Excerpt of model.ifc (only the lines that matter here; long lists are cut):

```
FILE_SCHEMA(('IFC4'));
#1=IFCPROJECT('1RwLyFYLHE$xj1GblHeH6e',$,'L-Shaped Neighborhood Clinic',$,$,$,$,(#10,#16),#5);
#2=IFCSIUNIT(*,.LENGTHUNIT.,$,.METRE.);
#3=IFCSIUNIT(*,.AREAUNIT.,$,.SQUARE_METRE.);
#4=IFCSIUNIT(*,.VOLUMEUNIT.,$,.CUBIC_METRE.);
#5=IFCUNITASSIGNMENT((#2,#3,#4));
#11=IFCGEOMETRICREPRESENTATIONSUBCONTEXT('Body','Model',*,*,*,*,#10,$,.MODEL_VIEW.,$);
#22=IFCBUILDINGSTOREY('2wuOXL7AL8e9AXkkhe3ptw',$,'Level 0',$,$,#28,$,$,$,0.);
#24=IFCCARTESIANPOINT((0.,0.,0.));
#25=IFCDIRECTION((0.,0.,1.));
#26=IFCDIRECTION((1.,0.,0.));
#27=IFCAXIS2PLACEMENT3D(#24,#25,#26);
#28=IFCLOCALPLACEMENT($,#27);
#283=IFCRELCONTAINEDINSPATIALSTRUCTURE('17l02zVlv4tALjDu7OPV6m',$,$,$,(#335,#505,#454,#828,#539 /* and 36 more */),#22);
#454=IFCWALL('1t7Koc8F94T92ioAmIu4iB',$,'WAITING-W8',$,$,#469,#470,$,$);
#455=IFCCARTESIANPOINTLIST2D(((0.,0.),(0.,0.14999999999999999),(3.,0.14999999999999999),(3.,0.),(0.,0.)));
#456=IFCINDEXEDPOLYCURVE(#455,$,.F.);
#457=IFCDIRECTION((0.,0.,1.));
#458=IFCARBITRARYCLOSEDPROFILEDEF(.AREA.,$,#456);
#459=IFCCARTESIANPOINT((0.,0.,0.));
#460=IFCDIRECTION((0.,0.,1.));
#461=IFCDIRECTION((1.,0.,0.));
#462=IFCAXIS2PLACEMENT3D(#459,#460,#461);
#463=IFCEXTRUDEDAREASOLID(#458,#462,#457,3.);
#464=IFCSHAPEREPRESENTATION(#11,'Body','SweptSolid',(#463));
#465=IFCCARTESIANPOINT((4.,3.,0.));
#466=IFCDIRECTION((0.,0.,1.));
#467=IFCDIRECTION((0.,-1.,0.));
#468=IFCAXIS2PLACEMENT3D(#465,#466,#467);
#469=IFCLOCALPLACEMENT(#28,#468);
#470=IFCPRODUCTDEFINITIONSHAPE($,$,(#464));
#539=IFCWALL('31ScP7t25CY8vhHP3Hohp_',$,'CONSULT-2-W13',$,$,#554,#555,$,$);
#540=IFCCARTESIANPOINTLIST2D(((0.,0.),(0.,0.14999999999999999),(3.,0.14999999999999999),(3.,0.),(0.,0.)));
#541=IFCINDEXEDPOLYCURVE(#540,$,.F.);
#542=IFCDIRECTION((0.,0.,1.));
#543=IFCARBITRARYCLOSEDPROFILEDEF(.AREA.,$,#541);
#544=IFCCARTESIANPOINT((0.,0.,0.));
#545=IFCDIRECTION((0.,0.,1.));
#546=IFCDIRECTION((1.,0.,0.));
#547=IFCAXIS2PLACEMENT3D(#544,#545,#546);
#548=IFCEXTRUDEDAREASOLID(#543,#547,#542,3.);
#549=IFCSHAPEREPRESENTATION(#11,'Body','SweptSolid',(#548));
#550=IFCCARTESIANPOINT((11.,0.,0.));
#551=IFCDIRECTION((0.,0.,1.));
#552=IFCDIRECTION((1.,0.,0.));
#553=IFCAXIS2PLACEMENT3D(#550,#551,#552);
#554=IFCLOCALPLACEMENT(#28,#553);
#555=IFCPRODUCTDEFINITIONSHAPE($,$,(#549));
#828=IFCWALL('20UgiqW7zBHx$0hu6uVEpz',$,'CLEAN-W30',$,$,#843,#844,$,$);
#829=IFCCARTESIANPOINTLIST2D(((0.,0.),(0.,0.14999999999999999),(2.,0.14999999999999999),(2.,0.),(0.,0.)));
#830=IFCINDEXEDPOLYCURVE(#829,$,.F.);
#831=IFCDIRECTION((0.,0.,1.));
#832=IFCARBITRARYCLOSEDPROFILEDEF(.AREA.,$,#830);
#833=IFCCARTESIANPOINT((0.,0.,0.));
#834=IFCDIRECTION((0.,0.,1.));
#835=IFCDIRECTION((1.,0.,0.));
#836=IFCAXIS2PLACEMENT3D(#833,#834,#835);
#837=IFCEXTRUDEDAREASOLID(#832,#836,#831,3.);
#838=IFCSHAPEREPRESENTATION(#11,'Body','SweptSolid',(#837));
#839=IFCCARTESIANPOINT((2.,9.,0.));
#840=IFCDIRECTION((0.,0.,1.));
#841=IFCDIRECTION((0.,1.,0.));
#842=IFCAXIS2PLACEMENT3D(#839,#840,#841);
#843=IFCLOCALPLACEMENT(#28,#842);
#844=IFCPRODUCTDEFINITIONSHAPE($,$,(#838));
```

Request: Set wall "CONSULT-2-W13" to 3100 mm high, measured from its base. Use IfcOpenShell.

```python
import ifcopenshell
import ifcopenshell.geom
import ifcopenshell.util.representation
import ifcopenshell.util.shape

model = ifcopenshell.open("model.ifc")
settings = ifcopenshell.geom.settings()


def volume(element):
    """Net volume in cubic metres, openings subtracted."""
    shape = ifcopenshell.geom.create_shape(settings, element)
    return ifcopenshell.util.shape.get_volume(shape.geometry)


wall = model.by_guid("31ScP7t25CY8vhHP3Hohp_")
before = volume(wall)

body = ifcopenshell.util.representation.get_representation(wall, "Model", "Body")
solid = body.Items[0]
old_height = solid.Depth
solid.Depth = 3.1
after = volume(wall)

print(f"height {old_height:g} -> {solid.Depth:g}, volume {before:.3f} -> {after:.3f} m3")

model.write("model-out.ifc")
```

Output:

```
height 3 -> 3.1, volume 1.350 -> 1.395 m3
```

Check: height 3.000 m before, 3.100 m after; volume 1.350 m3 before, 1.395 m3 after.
